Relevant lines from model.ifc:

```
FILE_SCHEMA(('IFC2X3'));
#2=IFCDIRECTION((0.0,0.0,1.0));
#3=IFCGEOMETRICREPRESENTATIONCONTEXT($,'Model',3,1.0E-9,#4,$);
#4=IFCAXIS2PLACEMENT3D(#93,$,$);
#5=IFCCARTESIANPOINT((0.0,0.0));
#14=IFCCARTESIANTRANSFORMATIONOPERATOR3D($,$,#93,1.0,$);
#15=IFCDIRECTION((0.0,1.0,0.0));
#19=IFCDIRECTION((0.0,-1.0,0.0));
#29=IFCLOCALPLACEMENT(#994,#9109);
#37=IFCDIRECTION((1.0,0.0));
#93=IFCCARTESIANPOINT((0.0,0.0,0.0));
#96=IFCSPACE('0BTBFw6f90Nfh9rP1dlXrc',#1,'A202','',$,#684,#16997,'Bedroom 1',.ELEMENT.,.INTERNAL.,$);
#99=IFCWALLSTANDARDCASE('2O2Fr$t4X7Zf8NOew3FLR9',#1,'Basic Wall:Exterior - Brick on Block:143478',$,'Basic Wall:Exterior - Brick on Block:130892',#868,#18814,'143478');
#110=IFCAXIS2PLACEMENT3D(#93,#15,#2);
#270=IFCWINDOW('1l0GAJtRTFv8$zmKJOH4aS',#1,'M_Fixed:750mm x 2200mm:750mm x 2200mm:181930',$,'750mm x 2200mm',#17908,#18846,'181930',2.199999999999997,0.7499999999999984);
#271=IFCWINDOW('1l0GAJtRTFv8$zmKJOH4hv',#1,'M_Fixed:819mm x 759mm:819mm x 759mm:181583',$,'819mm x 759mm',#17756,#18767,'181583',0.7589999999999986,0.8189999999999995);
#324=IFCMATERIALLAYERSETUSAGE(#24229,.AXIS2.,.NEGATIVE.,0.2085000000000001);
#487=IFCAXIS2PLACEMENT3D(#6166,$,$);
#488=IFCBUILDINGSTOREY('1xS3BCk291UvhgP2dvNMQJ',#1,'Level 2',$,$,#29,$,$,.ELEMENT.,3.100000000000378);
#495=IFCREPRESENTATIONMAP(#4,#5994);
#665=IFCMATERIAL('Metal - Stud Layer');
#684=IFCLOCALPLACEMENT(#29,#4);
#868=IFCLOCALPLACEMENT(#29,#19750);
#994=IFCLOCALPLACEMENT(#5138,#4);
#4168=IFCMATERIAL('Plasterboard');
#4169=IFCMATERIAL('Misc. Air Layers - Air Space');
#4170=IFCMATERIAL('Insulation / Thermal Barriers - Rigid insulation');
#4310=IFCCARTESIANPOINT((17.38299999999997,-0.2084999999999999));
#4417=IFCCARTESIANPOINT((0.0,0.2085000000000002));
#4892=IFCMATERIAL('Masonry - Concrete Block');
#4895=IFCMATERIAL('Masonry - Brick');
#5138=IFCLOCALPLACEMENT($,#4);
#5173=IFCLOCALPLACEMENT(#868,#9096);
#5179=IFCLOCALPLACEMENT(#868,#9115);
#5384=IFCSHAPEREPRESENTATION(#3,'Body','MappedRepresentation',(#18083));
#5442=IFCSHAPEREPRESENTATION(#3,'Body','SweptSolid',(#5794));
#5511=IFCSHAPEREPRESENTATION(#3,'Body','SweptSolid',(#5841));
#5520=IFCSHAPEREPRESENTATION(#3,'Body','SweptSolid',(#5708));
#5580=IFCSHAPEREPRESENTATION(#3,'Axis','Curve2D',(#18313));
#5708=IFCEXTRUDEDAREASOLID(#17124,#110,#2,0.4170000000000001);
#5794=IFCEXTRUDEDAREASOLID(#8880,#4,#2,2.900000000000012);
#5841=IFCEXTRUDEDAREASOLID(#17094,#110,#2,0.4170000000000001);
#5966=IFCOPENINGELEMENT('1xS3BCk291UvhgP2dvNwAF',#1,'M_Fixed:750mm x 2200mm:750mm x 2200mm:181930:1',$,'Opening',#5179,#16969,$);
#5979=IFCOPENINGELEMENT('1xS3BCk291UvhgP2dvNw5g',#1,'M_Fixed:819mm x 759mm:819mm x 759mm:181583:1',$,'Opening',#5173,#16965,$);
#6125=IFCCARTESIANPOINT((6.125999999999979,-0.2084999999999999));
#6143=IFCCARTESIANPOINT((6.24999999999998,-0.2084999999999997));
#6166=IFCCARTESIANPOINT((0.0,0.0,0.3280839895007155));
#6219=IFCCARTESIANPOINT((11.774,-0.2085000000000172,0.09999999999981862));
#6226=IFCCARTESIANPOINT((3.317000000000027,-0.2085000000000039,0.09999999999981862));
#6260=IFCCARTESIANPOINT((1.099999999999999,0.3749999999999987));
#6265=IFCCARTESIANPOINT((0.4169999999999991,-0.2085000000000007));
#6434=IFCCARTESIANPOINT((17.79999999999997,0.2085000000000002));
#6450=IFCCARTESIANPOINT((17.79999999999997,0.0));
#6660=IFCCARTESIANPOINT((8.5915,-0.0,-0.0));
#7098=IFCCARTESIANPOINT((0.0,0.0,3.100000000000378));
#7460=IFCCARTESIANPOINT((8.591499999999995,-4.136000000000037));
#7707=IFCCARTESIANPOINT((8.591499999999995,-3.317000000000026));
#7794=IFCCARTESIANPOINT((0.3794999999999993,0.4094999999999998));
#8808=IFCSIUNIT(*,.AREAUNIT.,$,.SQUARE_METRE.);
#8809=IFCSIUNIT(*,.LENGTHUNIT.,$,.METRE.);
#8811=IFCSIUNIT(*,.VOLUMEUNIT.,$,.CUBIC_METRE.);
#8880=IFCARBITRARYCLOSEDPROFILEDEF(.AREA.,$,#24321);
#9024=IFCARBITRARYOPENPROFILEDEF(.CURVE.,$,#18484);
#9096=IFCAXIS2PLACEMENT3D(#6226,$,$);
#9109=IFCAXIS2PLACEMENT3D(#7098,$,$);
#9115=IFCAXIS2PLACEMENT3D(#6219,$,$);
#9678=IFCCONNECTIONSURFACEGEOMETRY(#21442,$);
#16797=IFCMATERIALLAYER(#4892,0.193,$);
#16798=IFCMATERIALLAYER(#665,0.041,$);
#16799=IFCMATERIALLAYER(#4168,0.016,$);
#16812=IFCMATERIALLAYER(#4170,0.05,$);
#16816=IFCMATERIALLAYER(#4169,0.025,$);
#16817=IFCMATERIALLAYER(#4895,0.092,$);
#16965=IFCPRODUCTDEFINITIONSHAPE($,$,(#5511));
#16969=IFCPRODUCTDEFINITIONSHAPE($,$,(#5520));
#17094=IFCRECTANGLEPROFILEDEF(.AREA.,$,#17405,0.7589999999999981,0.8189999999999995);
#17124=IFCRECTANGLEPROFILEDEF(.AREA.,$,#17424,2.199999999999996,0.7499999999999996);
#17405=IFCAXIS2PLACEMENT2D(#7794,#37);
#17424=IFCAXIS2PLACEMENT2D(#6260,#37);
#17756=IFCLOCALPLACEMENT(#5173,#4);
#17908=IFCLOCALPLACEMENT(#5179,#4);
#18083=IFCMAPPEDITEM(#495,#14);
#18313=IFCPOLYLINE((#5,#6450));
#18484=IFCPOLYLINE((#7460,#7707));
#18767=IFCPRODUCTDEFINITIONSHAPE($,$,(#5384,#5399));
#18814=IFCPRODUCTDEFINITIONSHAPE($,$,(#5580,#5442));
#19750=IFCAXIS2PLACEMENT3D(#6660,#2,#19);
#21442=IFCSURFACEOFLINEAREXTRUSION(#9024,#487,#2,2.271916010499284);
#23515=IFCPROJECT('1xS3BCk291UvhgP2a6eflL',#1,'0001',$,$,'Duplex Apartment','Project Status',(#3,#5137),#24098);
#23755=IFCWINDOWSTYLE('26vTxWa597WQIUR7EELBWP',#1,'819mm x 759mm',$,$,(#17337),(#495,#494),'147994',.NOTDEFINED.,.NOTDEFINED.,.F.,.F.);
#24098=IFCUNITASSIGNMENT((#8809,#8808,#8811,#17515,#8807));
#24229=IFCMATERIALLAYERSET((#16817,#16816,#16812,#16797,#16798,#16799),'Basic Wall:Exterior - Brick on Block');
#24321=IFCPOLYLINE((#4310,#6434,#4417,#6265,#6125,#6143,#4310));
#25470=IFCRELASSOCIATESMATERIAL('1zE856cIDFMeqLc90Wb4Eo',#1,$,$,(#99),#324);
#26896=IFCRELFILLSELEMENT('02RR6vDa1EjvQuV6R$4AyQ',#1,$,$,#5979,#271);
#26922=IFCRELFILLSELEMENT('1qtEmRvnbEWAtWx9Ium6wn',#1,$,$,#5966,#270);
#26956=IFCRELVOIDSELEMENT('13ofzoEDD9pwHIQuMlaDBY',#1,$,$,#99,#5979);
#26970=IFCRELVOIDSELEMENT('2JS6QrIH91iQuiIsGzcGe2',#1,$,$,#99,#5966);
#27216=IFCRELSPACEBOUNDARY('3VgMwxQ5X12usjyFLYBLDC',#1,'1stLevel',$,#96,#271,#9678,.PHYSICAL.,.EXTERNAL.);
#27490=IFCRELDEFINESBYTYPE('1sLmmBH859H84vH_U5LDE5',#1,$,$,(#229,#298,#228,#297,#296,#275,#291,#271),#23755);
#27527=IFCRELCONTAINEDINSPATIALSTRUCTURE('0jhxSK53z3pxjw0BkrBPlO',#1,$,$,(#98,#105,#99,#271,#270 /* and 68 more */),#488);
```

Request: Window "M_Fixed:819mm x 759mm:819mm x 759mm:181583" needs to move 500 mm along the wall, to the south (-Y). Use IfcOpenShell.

```python
import numpy as np
import ifcopenshell
import ifcopenshell.api.geometry
import ifcopenshell.util.placement
import ifcopenshell.util.unit

model = ifcopenshell.open("model.ifc")
unit_scale = ifcopenshell.util.unit.calculate_unit_scale(model)

window = model.by_guid("1l0GAJtRTFv8$zmKJOH4hv")
opening = window.FillsVoids[0].RelatingOpeningElement
wall = opening.VoidsElements[0].RelatingBuildingElement

wall_matrix = ifcopenshell.util.placement.get_local_placement(wall.ObjectPlacement)
shift = wall_matrix[:3, 0] * 0.5 / unit_scale
before = ifcopenshell.util.placement.get_local_placement(window.ObjectPlacement)[:3, 3].copy()

# The window is placed relative to its opening, so it follows when the opening moves.
matrix = ifcopenshell.util.placement.get_local_placement(opening.ObjectPlacement)
matrix[:3, 3] += shift
ifcopenshell.api.geometry.edit_object_placement(
    model, product=opening, matrix=matrix, is_si=False, should_transform_children=True
)

# Space boundary surfaces are stored in each space's coordinates; move them too.
for rel in window.ProvidesBoundaries:
    if not rel.ConnectionGeometry:
        continue
    surface = rel.ConnectionGeometry.SurfaceOnRelatingElement
    space_matrix = ifcopenshell.util.placement.get_local_placement(rel.RelatingSpace.ObjectPlacement)
    point = np.array(surface.Position.Location.Coordinates) + space_matrix[:3, :3].T @ shift
    surface.Position = model.createIfcAxis2Placement3D(
        model.createIfcCartesianPoint(point.tolist()), surface.Position.Axis, surface.Position.RefDirection
    )

after = ifcopenshell.util.placement.get_local_placement(window.ObjectPlacement)[:3, 3]
print("window moved by", (after - before).round(3) + 0.0)

model.write("model-out.ifc")
```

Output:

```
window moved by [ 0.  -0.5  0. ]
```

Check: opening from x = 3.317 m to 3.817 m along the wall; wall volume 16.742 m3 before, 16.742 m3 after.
